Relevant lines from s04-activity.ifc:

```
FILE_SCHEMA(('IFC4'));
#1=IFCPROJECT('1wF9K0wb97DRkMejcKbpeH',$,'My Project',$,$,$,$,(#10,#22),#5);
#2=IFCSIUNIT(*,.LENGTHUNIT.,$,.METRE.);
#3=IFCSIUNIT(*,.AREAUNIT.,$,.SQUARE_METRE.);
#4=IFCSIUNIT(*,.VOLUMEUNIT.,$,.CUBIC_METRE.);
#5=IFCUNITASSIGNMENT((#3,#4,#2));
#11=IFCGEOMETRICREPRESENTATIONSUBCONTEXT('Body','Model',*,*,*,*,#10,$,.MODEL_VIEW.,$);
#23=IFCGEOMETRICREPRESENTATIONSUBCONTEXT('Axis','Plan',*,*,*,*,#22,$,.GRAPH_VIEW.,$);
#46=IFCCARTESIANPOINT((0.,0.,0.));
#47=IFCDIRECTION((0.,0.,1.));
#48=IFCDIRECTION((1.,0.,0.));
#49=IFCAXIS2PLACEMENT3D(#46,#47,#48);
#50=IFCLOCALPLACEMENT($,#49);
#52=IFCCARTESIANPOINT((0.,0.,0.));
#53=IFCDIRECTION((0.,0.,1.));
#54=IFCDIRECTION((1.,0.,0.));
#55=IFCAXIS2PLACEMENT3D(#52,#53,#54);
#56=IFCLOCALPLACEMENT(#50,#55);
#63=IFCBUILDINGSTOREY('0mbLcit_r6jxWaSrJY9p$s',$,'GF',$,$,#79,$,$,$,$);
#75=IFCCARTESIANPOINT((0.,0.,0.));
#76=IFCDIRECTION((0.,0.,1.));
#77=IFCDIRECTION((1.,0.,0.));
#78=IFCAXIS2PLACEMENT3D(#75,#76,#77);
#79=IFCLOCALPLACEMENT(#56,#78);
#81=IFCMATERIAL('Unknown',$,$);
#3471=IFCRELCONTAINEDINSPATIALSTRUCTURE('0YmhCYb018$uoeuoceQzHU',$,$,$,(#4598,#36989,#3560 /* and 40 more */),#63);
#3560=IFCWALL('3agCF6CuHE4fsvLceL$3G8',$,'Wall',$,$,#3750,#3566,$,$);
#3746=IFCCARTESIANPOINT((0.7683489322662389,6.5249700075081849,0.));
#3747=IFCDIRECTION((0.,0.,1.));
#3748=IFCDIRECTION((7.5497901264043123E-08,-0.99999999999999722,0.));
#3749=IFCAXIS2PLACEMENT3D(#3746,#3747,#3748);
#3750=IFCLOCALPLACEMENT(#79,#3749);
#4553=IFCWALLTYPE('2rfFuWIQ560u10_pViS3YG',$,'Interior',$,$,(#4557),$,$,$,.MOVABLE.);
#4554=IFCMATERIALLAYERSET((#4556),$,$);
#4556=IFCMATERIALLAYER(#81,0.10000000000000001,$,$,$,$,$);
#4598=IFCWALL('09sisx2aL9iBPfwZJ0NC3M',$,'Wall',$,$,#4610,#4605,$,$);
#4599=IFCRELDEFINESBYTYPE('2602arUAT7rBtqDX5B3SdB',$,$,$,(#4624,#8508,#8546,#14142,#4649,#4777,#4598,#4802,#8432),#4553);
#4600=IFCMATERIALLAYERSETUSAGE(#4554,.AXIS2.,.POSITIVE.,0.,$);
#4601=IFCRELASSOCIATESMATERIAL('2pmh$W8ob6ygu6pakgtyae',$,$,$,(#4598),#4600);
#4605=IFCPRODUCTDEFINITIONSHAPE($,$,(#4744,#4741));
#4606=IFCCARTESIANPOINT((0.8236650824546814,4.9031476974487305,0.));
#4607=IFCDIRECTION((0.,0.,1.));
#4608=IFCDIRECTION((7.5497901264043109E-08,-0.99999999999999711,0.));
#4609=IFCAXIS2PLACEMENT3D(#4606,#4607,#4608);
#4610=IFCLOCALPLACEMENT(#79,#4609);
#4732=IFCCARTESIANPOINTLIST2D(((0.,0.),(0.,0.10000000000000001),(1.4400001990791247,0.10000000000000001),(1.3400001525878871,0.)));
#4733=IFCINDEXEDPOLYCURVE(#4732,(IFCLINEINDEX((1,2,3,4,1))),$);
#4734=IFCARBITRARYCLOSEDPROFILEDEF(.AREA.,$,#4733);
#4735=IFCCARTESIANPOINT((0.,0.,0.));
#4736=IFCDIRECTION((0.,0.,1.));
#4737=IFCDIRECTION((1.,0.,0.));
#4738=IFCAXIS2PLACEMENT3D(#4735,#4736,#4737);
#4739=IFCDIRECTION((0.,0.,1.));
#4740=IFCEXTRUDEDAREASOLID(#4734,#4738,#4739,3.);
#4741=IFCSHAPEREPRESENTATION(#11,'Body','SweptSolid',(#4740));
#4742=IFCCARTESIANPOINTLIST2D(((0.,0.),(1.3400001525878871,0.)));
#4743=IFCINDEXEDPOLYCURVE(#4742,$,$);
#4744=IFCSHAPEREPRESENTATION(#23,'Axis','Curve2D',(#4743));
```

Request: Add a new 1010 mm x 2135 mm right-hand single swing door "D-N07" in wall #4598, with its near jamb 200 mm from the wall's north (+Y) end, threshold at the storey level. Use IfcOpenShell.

```python
import numpy as np
import ifcopenshell
import ifcopenshell.api.feature
import ifcopenshell.api.geometry
import ifcopenshell.api.root
import ifcopenshell.api.spatial
import ifcopenshell.geom
import ifcopenshell.util.element
import ifcopenshell.util.placement
import ifcopenshell.util.representation
import ifcopenshell.util.shape
import ifcopenshell.util.unit

model = ifcopenshell.open("s04-activity.ifc")
unit_scale = ifcopenshell.util.unit.calculate_unit_scale(model)
settings = ifcopenshell.geom.settings()


def volume(element):
    """Net volume in cubic metres, openings subtracted."""
    shape = ifcopenshell.geom.create_shape(settings, element)
    return ifcopenshell.util.shape.get_volume(shape.geometry)


wall = model.by_guid("09sisx2aL9iBPfwZJ0NC3M")
storey = ifcopenshell.util.element.get_container(wall, ifc_class="IfcBuildingStorey")
context = ifcopenshell.util.representation.get_context(model, "Model", "Body", "MODEL_VIEW")
before = volume(wall)

width, height, from_end, sill = 1.01, 2.135, 0.2, 0.0  # metres

# The wall runs along its own X axis, and the end named is its -X end.
wall_shape = ifcopenshell.geom.create_shape(settings, wall)
x, y, z = ifcopenshell.util.shape.get_vertices(wall_shape.geometry).T
start = x.min() + from_end
face, thickness = float(y.min()), float(y.max() - y.min())
wall_matrix = ifcopenshell.util.placement.get_local_placement(wall.ObjectPlacement)
level = ifcopenshell.util.placement.get_local_placement(storey.ObjectPlacement)[2, 3]


def in_wall(x, y):
    """Placement at x, y metres in the wall's axes, at sill height."""
    matrix = wall_matrix.copy()
    matrix[:, 3] = wall_matrix @ np.array([x / unit_scale, y / unit_scale, 0.0, 1.0])
    matrix[2, 3] = level + sill / unit_scale
    return matrix


# Opening: a box that overshoots both wall faces by 50 mm.
opening = ifcopenshell.api.root.create_entity(model, ifc_class="IfcOpeningElement", predefined_type="OPENING")
box = ifcopenshell.api.geometry.add_wall_representation(
    model, context=context, length=width, height=height, thickness=thickness + 0.1
)
ifcopenshell.api.geometry.assign_representation(model, product=opening, representation=box)
ifcopenshell.api.geometry.edit_object_placement(model, product=opening, matrix=in_wall(start, face - 0.05), is_si=False)
ifcopenshell.api.feature.add_feature(model, feature=opening, element=wall)

door = ifcopenshell.api.root.create_entity(model, ifc_class="IfcDoor", name="D-N07", predefined_type="DOOR")
door.OverallWidth, door.OverallHeight = width / unit_scale, height / unit_scale
door.OperationType = "SINGLE_SWING_RIGHT"
body = ifcopenshell.api.geometry.add_door_representation(
    model,
    context=context,
    overall_width=door.OverallWidth,
    overall_height=door.OverallHeight,
    operation_type="SINGLE_SWING_RIGHT",
    lining_properties={"LiningDepth": thickness / unit_scale, "ThresholdDepth": thickness / unit_scale},
)
ifcopenshell.api.geometry.assign_representation(model, product=door, representation=body)
ifcopenshell.api.spatial.assign_container(model, products=[door], relating_structure=storey)
ifcopenshell.api.feature.add_filling(model, opening=opening, element=door)

# The lining spans the wall, so the door starts at the wall face.
ifcopenshell.api.geometry.edit_object_placement(model, product=door, matrix=in_wall(start, face), is_si=False)

after = volume(wall)

print(f"wall volume {before:.3f} -> {after:.3f} m3")

model.write("s04-activity_updated.ifc")
```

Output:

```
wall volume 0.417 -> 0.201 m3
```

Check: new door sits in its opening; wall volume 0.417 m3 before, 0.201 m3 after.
